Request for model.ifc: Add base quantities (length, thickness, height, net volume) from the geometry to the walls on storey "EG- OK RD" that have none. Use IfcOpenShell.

First a look at what the model holds.

```python
import ifcopenshell
import ifcopenshell.util.element
import ifcopenshell.util.unit

model = ifcopenshell.open("model.ifc")
print(model.schema)
for unit_type in ("LENGTHUNIT", "AREAUNIT", "VOLUMEUNIT"):
    print(unit_type, ifcopenshell.util.unit.calculate_unit_scale(model, unit_type))
storey = next(s for s in model.by_type("IfcBuildingStorey") if s.Name == "EG- OK RD")
walls = [e for e in ifcopenshell.util.element.get_decomposition(storey) if e.is_a("IfcWall")]
for e in sorted(walls, key=lambda e: e.id()):
    print(e.id(), e.is_a(), e.Name, list(ifcopenshell.util.element.get_psets(e, qtos_only=True)), sep=" | ")
```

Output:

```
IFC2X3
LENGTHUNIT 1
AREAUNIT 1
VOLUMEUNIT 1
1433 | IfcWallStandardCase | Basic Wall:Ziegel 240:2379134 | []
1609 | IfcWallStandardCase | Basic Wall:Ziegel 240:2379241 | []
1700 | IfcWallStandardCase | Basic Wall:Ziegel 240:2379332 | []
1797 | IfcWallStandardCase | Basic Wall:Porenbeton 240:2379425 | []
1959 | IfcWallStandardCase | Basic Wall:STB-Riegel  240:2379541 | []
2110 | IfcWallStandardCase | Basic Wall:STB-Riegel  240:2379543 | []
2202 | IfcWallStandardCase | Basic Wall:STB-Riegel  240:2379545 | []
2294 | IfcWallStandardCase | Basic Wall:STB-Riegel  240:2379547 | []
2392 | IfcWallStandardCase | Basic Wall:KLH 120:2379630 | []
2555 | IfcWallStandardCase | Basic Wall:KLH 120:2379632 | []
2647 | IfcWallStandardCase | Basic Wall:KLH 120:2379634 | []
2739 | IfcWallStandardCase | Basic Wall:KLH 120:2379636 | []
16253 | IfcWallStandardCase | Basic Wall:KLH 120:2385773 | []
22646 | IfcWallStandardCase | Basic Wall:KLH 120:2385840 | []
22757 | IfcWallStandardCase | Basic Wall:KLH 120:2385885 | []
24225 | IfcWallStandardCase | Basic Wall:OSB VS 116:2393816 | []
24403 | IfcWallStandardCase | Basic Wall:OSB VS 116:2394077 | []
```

```python
import ifcopenshell
import ifcopenshell.api.pset
import ifcopenshell.geom
import ifcopenshell.util.element
import ifcopenshell.util.shape
import ifcopenshell.util.unit

model = ifcopenshell.open("model.ifc")
unit_scale = ifcopenshell.util.unit.calculate_unit_scale(model)
volume_scale = ifcopenshell.util.unit.calculate_unit_scale(model, "VOLUMEUNIT")
settings = ifcopenshell.geom.settings()

storey = next(s for s in model.by_type("IfcBuildingStorey") if s.Name == "EG- OK RD")
walls = [e for e in ifcopenshell.util.element.get_decomposition(storey) if e.is_a("IfcWall")]

for e in sorted(walls, key=lambda e: e.id()):
    if ifcopenshell.util.element.get_psets(e, qtos_only=True, should_inherit=False):
        continue
    # Geometry comes back in metres, in the element's own axes.
    shape = ifcopenshell.geom.create_shape(settings, e)
    values = {
        "Length": ifcopenshell.util.shape.get_x(shape.geometry) / unit_scale,
        "Width": ifcopenshell.util.shape.get_y(shape.geometry) / unit_scale,
        "Height": ifcopenshell.util.shape.get_z(shape.geometry) / unit_scale,
        "NetVolume": ifcopenshell.util.shape.get_volume(shape.geometry) / volume_scale,
    }
    qto = ifcopenshell.api.pset.add_qto(model, product=e, name="BaseQuantities")
    ifcopenshell.api.pset.edit_qto(model, qto=qto, properties=values)
    print(e.id(), {k: round(v, 3) for k, v in values.items()})

model.write("model_rev.ifc")
```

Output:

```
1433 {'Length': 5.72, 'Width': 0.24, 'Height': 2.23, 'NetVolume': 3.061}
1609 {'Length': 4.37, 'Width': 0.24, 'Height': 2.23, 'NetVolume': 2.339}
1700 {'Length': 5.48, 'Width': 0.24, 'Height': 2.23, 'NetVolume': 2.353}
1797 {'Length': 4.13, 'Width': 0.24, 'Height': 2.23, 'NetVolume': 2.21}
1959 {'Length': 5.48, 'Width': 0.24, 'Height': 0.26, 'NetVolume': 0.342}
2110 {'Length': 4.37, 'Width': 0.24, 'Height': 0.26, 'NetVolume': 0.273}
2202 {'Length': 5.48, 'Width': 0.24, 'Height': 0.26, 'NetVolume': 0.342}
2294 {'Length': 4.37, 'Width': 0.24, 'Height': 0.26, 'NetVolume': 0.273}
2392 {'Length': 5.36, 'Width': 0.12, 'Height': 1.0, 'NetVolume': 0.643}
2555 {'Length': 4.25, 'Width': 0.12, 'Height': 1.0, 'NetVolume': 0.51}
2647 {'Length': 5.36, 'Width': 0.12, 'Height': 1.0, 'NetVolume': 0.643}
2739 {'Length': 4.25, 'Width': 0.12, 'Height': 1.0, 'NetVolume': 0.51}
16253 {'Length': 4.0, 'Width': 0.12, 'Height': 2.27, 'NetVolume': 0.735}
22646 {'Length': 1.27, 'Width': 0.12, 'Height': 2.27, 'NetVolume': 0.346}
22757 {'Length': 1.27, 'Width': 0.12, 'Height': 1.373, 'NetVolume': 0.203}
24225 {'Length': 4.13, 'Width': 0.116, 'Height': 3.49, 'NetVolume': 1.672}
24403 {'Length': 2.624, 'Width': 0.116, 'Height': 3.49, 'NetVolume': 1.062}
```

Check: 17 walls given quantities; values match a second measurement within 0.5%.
